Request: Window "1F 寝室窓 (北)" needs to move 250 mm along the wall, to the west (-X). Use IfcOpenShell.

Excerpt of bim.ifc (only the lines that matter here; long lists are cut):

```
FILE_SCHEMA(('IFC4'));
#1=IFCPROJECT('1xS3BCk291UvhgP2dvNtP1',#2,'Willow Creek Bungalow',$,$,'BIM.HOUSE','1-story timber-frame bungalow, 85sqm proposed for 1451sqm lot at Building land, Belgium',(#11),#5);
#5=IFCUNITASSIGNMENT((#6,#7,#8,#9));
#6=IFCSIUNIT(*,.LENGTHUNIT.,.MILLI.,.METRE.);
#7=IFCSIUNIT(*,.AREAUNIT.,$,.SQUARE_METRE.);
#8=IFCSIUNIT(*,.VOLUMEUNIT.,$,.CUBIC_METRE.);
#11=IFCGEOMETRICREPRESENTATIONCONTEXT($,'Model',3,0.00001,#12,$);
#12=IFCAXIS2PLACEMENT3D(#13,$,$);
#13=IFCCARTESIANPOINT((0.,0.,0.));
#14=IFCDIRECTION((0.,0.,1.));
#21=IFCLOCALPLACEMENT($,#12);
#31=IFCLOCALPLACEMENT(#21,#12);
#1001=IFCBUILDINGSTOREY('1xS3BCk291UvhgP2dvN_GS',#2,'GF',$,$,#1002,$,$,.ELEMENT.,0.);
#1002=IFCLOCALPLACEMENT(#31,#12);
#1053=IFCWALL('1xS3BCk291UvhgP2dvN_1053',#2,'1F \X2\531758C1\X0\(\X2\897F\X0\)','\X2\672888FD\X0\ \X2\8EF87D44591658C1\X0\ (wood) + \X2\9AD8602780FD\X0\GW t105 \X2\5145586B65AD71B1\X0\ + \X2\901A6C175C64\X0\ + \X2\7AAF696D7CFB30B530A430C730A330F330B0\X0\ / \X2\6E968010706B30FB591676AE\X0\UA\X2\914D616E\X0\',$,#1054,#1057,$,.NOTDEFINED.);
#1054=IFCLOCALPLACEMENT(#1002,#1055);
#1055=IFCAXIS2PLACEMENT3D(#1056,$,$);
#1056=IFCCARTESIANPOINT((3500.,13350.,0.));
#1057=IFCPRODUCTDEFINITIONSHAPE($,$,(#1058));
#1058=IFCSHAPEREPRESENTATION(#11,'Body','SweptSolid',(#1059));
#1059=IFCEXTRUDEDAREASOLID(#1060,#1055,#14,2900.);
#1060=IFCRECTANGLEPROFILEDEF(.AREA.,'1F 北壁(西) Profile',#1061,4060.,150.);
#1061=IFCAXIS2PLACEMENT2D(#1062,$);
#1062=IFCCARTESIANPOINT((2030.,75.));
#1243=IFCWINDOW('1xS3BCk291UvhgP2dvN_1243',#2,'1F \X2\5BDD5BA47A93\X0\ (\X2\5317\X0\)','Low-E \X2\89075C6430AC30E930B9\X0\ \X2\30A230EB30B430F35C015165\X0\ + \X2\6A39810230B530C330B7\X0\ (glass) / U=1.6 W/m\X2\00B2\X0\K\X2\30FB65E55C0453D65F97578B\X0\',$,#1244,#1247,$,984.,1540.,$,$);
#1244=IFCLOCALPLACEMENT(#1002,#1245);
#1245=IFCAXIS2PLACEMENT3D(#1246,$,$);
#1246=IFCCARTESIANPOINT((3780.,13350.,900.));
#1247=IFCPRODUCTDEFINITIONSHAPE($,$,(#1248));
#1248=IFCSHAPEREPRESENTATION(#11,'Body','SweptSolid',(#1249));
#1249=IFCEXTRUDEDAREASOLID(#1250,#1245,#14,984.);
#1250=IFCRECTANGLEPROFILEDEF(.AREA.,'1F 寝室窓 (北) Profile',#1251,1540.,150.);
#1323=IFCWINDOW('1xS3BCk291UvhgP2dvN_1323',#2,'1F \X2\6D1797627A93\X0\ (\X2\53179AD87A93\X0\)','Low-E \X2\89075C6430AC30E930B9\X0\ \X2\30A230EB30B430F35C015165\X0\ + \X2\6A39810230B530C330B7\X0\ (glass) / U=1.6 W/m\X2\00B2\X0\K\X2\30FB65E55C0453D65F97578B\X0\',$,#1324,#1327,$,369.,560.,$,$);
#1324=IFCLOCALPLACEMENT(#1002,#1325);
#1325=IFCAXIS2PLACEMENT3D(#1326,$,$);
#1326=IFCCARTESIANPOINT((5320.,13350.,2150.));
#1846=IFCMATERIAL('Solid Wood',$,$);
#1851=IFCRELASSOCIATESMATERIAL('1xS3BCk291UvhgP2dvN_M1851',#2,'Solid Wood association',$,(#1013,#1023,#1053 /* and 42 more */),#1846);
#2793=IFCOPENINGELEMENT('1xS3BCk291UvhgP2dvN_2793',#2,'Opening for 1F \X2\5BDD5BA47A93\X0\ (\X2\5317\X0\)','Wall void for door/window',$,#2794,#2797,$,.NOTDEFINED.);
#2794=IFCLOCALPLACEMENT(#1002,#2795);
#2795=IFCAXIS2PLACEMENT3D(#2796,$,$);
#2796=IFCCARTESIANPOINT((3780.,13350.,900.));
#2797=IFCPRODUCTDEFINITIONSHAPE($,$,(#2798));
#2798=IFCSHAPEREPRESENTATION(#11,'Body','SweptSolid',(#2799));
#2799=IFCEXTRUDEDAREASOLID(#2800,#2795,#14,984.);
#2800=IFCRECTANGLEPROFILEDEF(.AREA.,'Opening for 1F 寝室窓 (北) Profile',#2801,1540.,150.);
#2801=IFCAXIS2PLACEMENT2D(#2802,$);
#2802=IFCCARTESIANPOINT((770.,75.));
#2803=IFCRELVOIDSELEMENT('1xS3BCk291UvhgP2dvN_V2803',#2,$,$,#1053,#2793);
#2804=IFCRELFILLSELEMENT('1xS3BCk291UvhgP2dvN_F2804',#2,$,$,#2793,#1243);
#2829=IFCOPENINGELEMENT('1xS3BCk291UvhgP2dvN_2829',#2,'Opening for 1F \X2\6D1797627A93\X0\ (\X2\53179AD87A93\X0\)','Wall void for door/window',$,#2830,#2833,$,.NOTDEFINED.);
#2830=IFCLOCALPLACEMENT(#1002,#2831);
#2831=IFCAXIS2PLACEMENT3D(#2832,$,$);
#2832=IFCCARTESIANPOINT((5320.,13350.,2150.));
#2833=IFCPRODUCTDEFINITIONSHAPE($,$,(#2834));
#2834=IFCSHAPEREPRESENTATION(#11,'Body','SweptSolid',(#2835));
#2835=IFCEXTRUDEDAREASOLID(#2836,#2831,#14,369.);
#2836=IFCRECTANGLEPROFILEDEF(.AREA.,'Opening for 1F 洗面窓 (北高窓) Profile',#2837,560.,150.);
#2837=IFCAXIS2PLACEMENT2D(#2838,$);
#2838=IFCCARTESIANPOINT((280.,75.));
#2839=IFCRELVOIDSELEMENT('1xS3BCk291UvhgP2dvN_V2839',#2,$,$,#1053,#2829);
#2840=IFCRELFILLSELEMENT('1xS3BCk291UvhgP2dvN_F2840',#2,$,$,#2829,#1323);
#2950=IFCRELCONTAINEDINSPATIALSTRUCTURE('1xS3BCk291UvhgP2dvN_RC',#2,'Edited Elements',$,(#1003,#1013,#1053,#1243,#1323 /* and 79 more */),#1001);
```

```python
import ifcopenshell
import ifcopenshell.api.geometry
import ifcopenshell.util.placement
import ifcopenshell.util.unit

model = ifcopenshell.open("bim.ifc")
unit_scale = ifcopenshell.util.unit.calculate_unit_scale(model)

window = model.by_id(1243)
opening = window.FillsVoids[0].RelatingOpeningElement
wall = opening.VoidsElements[0].RelatingBuildingElement

wall_matrix = ifcopenshell.util.placement.get_local_placement(wall.ObjectPlacement)
shift = wall_matrix[:3, 0] * -0.25 / unit_scale
before = ifcopenshell.util.placement.get_local_placement(window.ObjectPlacement)[:3, 3].copy()

# The window is not placed relative to its opening, so move both.
for product in (opening, window):
    matrix = ifcopenshell.util.placement.get_local_placement(product.ObjectPlacement)
    matrix[:3, 3] += shift
    ifcopenshell.api.geometry.edit_object_placement(model, product=product, matrix=matrix, is_si=False)

after = ifcopenshell.util.placement.get_local_placement(window.ObjectPlacement)[:3, 3]
print("window moved by", (after - before).round(3) + 0.0)

model.write("bim_updated.ifc")
```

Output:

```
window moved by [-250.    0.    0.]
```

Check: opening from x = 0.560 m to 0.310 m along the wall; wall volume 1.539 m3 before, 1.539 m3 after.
